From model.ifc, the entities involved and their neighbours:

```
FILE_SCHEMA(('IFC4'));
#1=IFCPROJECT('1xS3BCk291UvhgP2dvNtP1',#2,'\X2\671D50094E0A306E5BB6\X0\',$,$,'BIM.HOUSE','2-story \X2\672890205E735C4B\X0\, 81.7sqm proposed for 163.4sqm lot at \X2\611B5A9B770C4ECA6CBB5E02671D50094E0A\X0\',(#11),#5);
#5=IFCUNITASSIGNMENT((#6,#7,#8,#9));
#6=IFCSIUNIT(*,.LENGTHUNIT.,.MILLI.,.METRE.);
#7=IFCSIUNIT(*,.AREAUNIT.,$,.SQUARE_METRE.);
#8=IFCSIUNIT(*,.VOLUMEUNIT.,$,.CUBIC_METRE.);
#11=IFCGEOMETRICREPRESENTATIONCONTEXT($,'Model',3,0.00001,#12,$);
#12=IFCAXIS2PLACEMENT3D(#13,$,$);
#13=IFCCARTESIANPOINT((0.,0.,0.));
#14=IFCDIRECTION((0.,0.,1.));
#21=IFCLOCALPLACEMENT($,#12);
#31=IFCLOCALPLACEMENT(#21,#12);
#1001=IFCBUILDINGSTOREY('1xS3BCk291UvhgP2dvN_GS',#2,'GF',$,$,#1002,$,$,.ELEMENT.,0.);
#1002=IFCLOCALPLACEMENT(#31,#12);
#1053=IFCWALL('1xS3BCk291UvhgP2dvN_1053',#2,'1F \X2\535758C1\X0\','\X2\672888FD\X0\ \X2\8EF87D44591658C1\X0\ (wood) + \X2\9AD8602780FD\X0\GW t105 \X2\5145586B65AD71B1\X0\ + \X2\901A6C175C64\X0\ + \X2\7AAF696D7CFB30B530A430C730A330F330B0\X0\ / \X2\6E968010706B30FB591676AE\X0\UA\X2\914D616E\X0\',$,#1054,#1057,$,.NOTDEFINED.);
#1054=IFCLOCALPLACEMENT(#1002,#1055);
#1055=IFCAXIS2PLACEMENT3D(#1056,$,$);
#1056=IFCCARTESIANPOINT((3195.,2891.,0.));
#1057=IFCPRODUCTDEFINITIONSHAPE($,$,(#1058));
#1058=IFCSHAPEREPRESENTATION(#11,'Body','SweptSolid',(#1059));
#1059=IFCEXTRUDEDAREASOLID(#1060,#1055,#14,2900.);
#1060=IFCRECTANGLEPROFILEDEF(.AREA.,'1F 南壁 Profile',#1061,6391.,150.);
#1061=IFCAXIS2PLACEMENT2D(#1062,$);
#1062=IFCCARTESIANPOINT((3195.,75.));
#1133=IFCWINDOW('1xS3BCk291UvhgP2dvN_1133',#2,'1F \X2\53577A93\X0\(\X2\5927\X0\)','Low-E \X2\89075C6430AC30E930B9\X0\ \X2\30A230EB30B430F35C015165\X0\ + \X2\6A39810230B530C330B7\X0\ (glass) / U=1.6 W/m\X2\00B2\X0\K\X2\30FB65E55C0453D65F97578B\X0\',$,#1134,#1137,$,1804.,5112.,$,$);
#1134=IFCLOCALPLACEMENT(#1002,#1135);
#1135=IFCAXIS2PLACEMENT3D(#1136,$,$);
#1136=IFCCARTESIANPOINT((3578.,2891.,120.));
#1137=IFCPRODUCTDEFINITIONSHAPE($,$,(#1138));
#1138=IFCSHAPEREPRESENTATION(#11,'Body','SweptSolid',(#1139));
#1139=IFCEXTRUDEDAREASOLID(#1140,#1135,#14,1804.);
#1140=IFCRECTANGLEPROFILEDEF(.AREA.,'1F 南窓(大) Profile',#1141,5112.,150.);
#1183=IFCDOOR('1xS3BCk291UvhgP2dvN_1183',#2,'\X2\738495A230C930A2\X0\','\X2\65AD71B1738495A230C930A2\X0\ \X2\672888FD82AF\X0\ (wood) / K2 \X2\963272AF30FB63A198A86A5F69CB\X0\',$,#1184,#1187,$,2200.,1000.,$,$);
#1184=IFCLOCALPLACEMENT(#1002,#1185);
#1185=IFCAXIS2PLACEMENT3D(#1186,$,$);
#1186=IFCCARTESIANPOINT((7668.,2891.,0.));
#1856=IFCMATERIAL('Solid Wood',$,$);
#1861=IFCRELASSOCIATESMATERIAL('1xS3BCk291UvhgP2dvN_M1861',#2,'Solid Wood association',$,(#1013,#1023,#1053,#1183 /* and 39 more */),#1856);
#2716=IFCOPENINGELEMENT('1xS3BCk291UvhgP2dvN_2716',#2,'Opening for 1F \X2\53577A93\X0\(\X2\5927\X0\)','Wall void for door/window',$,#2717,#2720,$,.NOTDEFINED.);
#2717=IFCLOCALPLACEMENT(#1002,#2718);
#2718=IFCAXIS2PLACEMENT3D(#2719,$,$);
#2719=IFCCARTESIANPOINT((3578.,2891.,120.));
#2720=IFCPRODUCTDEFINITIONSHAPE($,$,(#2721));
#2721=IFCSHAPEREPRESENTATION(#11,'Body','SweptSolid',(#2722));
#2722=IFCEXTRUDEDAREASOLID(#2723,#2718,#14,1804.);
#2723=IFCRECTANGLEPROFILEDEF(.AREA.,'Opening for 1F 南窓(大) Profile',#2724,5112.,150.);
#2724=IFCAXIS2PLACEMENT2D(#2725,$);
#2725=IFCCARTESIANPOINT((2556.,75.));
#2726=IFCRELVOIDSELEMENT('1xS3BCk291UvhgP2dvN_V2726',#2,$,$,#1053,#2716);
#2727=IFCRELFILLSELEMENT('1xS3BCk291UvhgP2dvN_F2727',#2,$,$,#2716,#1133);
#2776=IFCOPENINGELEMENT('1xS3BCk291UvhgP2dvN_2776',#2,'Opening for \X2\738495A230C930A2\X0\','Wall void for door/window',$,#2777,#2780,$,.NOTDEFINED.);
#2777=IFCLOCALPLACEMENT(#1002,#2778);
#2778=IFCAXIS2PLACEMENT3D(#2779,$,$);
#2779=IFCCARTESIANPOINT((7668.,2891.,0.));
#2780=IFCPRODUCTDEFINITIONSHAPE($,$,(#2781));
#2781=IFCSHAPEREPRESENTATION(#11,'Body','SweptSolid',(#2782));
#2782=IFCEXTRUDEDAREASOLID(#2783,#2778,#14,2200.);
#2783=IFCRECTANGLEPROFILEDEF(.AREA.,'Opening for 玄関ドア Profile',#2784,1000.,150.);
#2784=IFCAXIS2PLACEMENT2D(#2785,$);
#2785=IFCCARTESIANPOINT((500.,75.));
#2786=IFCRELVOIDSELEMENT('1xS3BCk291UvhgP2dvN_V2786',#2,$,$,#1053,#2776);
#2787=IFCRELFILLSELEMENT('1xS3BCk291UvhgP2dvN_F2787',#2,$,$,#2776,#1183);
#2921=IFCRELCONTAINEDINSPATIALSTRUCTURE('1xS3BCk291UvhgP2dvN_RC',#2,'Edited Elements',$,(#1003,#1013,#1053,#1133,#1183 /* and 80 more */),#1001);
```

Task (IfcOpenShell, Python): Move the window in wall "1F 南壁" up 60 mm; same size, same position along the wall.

```python
import numpy as np
import ifcopenshell
import ifcopenshell.api.geometry
import ifcopenshell.util.placement
import ifcopenshell.util.unit

model = ifcopenshell.open("model.ifc")
unit_scale = ifcopenshell.util.unit.calculate_unit_scale(model)

window = model.by_guid("1xS3BCk291UvhgP2dvN_1133")
opening = window.FillsVoids[0].RelatingOpeningElement
dz = 0.06 / unit_scale

shift = np.array([0.0, 0.0, dz])
# The window is not placed relative to its opening, so move both.
for product in (opening, window):
    matrix = ifcopenshell.util.placement.get_local_placement(product.ObjectPlacement)
    matrix[:3, 3] += shift
    ifcopenshell.api.geometry.edit_object_placement(model, product=product, matrix=matrix, is_si=False)

print(f"moved by {dz * unit_scale:+.3f} m")

model.write("model_rev.ifc")
```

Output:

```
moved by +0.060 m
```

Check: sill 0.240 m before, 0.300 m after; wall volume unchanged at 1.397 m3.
